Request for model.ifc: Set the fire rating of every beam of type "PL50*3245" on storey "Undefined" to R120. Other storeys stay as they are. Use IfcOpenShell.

First a look at what the model holds.

```python
import ifcopenshell
import ifcopenshell.util.element

model = ifcopenshell.open("model.ifc")
print(model.schema)
storey = next(s for s in model.by_type("IfcBuildingStorey") if s.Name == "Undefined")
beams = [e for e in ifcopenshell.util.element.get_decomposition(storey) if e.is_a("IfcBeam")]
seen = {}
for e in beams:
    element_type = ifcopenshell.util.element.get_type(e)
    key = (element_type.Name if element_type != e and element_type else None, ifcopenshell.util.element.get_pset(e, "Pset_BeamCommon", "FireRating"))
    seen[key] = seen.get(key, 0) + 1
for (name, value), count in sorted(seen.items(), key=str):
    print(count, "x", name, "|", value)
```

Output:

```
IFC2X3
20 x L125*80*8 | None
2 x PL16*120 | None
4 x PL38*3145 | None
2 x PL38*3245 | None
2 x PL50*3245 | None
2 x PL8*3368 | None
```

```python
import ifcopenshell
import ifcopenshell.api.pset
import ifcopenshell.util.element

model = ifcopenshell.open("model.ifc")

storey = next(s for s in model.by_type("IfcBuildingStorey") if s.Name == "Undefined")
beams = [e for e in ifcopenshell.util.element.get_decomposition(storey) if e.is_a("IfcBeam")]

count = 0
for e in beams:
    element_type = ifcopenshell.util.element.get_type(e)
    if element_type in (None, e) or element_type.Name != "PL50*3245":
        continue
    # add_pset returns the element's existing set when there is one.
    pset = ifcopenshell.api.pset.add_pset(model, product=e, name="Pset_BeamCommon")
    ifcopenshell.api.pset.edit_pset(model, pset=pset, properties={"FireRating": "R120"})
    count += 1

print(count, "beams updated")

model.write("model_edited.ifc")
```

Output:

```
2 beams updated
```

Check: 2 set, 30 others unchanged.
